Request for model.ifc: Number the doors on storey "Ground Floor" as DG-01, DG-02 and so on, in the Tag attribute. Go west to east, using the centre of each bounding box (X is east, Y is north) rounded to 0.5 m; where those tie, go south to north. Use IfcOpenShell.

First a look at what the model holds.

```python
import ifcopenshell
import ifcopenshell.util.element
import ifcopenshell.util.placement

model = ifcopenshell.open("model.ifc")
print(model.schema)
storey = next(s for s in model.by_type("IfcBuildingStorey") if s.Name == "Ground Floor")
doors = [e for e in ifcopenshell.util.element.get_decomposition(storey) if e.is_a("IfcDoor")]
for e in sorted(doors, key=lambda e: e.id()):
    origin = ifcopenshell.util.placement.get_local_placement(e.ObjectPlacement)[:3, 3]
    print(e.id(), e.Tag, e.Name, origin.round(2) + 0.0, sep=" | ")
```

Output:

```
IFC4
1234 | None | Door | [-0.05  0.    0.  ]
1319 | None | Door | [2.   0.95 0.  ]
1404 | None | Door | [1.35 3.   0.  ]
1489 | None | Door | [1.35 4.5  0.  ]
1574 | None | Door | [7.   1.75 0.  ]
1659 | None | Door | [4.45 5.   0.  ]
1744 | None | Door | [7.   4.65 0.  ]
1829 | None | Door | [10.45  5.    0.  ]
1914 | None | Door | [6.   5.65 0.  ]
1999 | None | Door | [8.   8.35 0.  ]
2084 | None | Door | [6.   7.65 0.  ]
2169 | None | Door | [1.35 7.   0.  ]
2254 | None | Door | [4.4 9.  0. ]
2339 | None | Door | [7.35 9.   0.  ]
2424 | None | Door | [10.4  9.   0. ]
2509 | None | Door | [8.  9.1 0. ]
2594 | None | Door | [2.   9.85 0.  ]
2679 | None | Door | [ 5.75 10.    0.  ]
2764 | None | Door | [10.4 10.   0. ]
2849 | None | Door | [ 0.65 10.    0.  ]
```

```python
import ifcopenshell
import ifcopenshell.geom
import ifcopenshell.util.element
import ifcopenshell.util.shape

model = ifcopenshell.open("model.ifc")
settings = ifcopenshell.geom.settings()
settings.set("use-world-coords", True)


def centre(element):
    shape = ifcopenshell.geom.create_shape(settings, element)
    return ifcopenshell.util.shape.get_bbox_centroid(shape.geometry)


storey = next(s for s in model.by_type("IfcBuildingStorey") if s.Name == "Ground Floor")
doors = [e for e in ifcopenshell.util.element.get_decomposition(storey) if e.is_a("IfcDoor")]

# Insertion points can sit at a corner or the storey origin, so sort by the geometry (in metres).
centres = {e: centre(e) for e in doors}
doors.sort(key=lambda e: (round(centres[e][0] / 0.5), centres[e][1]))

for i, e in enumerate(doors, start=1):
    number = f"DG-{i:02d}"
    e.Tag = number
    print(e.id(), number)

model.write("model_edited.ifc")
```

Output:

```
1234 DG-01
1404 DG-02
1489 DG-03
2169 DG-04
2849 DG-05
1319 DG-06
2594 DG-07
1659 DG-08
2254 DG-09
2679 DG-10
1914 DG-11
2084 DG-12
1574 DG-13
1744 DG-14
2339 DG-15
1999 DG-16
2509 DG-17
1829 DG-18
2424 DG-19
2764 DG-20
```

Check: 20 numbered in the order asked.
